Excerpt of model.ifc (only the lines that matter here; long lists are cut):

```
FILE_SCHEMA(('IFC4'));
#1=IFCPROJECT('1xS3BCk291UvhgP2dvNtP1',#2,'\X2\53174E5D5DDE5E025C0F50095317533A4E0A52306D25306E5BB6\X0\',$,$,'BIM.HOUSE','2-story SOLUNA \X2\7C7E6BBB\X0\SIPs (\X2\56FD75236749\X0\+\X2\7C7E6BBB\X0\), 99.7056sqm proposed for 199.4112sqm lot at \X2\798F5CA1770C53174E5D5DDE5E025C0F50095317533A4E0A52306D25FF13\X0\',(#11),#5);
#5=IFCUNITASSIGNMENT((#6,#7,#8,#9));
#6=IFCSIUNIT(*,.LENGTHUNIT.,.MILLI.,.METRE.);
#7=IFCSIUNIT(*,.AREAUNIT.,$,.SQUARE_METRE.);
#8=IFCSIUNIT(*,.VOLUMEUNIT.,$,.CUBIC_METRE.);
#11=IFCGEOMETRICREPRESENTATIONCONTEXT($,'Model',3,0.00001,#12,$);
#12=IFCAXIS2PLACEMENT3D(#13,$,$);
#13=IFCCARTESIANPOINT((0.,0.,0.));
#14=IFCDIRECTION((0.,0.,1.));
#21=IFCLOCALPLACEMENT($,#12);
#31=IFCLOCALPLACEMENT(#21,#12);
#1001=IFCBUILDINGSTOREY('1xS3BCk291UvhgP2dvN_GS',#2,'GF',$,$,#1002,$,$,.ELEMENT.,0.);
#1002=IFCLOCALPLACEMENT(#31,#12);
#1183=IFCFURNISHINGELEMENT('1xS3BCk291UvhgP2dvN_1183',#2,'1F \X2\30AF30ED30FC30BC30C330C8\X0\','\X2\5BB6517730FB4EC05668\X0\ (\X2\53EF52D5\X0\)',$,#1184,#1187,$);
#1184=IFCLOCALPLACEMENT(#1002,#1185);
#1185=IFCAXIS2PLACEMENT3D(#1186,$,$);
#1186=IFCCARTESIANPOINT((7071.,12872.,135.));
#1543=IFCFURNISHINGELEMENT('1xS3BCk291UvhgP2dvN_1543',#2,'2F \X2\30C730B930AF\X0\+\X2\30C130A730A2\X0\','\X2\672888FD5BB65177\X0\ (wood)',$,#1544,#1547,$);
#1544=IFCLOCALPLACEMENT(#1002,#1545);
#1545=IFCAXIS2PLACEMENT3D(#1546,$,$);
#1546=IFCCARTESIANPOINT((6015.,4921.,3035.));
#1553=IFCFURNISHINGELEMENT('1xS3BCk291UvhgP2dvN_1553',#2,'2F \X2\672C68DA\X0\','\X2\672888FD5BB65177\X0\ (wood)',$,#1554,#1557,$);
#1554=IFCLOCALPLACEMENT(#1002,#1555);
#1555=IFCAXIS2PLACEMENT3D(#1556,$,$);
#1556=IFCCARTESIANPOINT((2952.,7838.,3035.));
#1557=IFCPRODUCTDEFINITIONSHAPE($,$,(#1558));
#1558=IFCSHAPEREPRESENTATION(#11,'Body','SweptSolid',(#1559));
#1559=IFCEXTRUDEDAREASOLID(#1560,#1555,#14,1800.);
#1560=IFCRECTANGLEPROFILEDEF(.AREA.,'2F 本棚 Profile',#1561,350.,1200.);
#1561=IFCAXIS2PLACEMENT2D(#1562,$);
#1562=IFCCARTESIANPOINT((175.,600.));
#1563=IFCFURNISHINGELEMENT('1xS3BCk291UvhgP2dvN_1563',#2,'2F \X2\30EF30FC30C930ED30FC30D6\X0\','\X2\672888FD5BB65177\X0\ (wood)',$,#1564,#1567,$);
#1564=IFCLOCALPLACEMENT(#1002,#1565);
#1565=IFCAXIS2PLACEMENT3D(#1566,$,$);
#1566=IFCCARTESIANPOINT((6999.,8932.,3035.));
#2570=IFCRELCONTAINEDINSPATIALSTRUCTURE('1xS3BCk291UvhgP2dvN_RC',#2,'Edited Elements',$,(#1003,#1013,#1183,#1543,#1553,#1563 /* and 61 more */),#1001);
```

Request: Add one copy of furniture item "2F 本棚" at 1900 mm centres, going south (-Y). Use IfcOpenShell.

```python
import numpy as np
import ifcopenshell
import ifcopenshell.api.geometry
import ifcopenshell.api.root
import ifcopenshell.util.element
import ifcopenshell.util.placement

model = ifcopenshell.open("model.ifc")


def reuse_history(source, copy):
    """copy_class also copies each property set's owner history, people and application; keep the originals."""
    for rel in copy.IsDefinedBy:
        if rel.is_a("IfcRelDefinesByProperties") and (history := rel.RelatingPropertyDefinition.OwnerHistory):
            rel.RelatingPropertyDefinition.OwnerHistory = source.OwnerHistory
            ifcopenshell.util.element.remove_deep2(model, history)


source = model.by_guid("1xS3BCk291UvhgP2dvN_1553")
base = ifcopenshell.util.placement.get_local_placement(source.ObjectPlacement)
step = np.array([0.0, -1.0, 0.0]) * 1900.0

for i in range(1, 2):
    copy = ifcopenshell.api.root.copy_class(model, product=source)
    copy.Representation = ifcopenshell.util.element.copy_deep(
        model, source.Representation, exclude=["IfcGeometricRepresentationContext", "IfcRepresentationMap"]
    )
    reuse_history(source, copy)
    matrix = base.copy()
    matrix[:3, 3] += i * step
    print("added at", matrix[:3, 3].round(3) + 0.0)
    ifcopenshell.api.geometry.edit_object_placement(model, product=copy, matrix=matrix, is_si=False)

model.write("model-out.ifc")
```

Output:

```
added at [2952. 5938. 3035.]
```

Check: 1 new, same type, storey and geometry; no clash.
